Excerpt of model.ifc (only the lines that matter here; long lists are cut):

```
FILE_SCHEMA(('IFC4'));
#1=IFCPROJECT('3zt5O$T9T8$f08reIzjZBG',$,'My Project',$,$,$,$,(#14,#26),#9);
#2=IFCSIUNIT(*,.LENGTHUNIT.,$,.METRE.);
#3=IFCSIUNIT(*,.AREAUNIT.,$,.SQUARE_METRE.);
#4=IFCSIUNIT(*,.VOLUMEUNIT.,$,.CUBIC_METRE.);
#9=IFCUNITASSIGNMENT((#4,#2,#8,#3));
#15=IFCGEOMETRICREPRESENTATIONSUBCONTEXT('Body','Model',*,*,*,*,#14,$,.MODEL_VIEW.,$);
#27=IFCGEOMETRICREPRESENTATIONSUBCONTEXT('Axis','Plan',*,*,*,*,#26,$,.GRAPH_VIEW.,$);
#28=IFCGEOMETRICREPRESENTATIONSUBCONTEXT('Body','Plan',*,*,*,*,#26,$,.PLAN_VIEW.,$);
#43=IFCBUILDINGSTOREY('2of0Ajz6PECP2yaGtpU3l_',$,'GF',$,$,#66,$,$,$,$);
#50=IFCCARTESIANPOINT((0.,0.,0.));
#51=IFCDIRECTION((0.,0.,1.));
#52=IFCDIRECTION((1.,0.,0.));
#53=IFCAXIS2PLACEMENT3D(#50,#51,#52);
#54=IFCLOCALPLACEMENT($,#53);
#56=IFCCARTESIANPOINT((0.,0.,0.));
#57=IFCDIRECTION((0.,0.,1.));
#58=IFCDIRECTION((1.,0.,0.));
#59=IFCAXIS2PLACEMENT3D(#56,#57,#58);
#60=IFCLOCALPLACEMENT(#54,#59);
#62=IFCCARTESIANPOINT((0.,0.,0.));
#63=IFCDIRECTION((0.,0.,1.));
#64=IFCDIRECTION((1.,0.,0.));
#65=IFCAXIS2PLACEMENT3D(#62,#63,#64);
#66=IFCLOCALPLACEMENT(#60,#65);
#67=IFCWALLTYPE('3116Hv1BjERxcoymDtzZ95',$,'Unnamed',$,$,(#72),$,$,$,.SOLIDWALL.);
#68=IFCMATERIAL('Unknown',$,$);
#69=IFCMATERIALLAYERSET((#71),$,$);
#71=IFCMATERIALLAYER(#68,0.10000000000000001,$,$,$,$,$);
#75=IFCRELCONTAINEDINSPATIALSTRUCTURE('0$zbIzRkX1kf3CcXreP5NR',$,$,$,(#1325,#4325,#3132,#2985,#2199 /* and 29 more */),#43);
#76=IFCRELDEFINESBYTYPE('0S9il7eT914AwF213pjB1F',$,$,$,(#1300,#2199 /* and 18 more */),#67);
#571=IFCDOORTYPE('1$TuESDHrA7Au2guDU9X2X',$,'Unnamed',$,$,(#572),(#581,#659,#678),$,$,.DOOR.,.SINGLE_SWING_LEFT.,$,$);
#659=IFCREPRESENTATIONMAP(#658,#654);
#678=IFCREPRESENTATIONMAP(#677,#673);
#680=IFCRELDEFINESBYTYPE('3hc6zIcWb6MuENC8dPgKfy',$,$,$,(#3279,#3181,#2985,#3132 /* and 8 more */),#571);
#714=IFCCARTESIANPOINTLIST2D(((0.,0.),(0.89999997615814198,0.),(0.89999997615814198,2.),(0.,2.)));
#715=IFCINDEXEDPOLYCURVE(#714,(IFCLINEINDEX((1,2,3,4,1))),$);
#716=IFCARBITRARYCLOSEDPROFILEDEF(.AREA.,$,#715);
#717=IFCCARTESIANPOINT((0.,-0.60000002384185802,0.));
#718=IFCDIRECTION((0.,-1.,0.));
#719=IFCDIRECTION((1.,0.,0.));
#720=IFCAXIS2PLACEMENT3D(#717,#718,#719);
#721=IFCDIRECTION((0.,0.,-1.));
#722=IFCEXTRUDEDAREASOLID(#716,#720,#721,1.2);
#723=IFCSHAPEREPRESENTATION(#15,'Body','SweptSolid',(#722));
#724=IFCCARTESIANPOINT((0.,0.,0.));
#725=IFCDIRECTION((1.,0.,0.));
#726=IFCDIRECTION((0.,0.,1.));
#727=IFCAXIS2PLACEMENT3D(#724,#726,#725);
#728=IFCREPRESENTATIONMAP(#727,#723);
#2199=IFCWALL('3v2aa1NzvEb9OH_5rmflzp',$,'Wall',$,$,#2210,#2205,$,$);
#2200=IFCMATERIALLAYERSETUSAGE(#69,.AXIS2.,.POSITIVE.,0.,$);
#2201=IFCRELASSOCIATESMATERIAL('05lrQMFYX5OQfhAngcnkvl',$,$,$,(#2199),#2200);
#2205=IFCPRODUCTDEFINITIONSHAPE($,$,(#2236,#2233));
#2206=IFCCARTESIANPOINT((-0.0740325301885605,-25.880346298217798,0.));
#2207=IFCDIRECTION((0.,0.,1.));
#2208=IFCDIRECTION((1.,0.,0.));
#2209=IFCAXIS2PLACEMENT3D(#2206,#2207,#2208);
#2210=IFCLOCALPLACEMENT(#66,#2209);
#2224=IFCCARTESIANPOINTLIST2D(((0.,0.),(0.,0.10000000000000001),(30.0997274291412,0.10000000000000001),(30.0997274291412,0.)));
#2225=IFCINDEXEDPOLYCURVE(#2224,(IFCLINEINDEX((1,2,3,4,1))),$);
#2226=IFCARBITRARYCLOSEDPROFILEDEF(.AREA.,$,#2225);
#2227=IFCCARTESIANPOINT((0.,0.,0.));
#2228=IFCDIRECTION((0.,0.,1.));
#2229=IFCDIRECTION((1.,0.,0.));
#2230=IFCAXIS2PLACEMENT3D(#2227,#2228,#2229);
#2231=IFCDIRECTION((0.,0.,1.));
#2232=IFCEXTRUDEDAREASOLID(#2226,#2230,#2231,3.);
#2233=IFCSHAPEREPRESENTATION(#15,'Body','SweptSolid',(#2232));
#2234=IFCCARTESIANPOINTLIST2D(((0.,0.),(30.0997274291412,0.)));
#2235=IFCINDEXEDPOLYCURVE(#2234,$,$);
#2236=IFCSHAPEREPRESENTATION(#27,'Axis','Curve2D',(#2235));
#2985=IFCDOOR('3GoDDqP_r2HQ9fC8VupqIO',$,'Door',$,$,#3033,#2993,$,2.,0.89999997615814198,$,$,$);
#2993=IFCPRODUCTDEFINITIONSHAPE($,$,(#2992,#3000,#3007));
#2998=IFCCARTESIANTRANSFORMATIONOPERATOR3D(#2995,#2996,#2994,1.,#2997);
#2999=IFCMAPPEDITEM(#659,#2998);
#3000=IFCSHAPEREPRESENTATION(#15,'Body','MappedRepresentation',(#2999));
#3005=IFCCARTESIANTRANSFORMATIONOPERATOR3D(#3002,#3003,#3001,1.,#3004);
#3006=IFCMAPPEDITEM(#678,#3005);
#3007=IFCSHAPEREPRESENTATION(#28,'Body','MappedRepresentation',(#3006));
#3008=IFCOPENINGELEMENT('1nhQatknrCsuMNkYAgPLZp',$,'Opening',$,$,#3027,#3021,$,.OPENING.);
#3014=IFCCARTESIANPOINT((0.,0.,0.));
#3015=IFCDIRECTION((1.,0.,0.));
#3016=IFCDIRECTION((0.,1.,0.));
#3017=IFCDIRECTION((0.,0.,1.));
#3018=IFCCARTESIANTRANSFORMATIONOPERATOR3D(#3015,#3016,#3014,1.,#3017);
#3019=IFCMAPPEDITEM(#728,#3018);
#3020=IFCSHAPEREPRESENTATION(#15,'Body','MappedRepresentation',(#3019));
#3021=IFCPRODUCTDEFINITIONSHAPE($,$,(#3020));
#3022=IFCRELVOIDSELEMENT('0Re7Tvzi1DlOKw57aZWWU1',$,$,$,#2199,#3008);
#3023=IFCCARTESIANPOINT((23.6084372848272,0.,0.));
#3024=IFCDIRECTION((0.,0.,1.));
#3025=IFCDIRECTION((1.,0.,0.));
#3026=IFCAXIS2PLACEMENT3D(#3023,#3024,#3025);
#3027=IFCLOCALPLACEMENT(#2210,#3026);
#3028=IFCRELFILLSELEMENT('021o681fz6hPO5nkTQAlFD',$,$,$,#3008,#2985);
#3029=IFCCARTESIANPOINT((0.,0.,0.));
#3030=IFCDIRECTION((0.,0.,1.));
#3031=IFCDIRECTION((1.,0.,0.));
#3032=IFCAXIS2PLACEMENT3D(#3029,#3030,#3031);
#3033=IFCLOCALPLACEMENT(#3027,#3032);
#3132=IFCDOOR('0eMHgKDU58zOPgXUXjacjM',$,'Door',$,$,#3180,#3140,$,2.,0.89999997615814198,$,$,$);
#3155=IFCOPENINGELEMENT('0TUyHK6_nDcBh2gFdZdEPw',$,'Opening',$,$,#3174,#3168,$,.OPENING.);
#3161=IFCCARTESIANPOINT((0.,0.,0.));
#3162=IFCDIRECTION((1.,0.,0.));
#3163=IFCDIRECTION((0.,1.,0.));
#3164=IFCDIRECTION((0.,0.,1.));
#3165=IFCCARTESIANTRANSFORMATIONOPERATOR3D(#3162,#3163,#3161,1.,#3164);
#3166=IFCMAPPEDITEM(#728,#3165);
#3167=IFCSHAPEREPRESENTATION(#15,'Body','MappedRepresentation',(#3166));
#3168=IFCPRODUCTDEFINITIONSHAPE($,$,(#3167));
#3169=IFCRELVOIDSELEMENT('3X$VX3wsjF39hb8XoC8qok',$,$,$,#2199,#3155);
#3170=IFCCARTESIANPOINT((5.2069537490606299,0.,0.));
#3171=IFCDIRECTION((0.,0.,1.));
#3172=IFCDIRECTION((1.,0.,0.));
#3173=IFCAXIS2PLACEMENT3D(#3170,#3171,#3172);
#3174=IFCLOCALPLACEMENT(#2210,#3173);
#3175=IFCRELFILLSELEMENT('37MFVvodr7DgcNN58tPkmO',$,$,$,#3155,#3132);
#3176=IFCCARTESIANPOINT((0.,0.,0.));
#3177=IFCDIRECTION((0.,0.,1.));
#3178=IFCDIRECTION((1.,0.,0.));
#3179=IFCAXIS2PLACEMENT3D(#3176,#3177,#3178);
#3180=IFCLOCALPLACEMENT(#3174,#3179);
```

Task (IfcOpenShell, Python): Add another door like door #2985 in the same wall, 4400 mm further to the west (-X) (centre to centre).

```python
import ifcopenshell
import ifcopenshell.api.feature
import ifcopenshell.api.geometry
import ifcopenshell.api.root
import ifcopenshell.geom
import ifcopenshell.util.element
import ifcopenshell.util.placement
import ifcopenshell.util.shape
import ifcopenshell.util.unit

model = ifcopenshell.open("model.ifc")
unit_scale = ifcopenshell.util.unit.calculate_unit_scale(model)
settings = ifcopenshell.geom.settings()


def volume(element):
    """Net volume in cubic metres, openings subtracted."""
    shape = ifcopenshell.geom.create_shape(settings, element)
    return ifcopenshell.util.shape.get_volume(shape.geometry)


door = model.by_guid("3GoDDqP_r2HQ9fC8VupqIO")
opening = door.FillsVoids[0].RelatingOpeningElement
wall = opening.VoidsElements[0].RelatingBuildingElement
before = volume(wall)
shift = ifcopenshell.util.placement.get_local_placement(wall.ObjectPlacement)[:3, 0] * -4.4 / unit_scale

# copy_class copies the void relationship, type, container and properties, but no geometry.
new_opening = ifcopenshell.api.root.copy_class(model, product=opening)
new_opening.Representation = ifcopenshell.util.element.copy_deep(
    model, opening.Representation, exclude=["IfcGeometricRepresentationContext", "IfcRepresentationMap"]
)
new_door = ifcopenshell.api.root.copy_class(model, product=door)
new_door.Representation = ifcopenshell.util.element.copy_deep(
    model, door.Representation, exclude=["IfcGeometricRepresentationContext", "IfcRepresentationMap"]
)
ifcopenshell.api.feature.add_filling(model, opening=new_opening, element=new_door)

for old, new in ((opening, new_opening), (door, new_door)):
    matrix = ifcopenshell.util.placement.get_local_placement(old.ObjectPlacement)
    matrix[:3, 3] += shift
    ifcopenshell.api.geometry.edit_object_placement(model, product=new, matrix=matrix, is_si=False)

after = volume(wall)

print(f"wall volume {before:.3f} -> {after:.3f} m3")

model.write("model_rev.ifc")
```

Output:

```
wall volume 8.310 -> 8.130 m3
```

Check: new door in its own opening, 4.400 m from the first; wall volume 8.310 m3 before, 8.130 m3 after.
